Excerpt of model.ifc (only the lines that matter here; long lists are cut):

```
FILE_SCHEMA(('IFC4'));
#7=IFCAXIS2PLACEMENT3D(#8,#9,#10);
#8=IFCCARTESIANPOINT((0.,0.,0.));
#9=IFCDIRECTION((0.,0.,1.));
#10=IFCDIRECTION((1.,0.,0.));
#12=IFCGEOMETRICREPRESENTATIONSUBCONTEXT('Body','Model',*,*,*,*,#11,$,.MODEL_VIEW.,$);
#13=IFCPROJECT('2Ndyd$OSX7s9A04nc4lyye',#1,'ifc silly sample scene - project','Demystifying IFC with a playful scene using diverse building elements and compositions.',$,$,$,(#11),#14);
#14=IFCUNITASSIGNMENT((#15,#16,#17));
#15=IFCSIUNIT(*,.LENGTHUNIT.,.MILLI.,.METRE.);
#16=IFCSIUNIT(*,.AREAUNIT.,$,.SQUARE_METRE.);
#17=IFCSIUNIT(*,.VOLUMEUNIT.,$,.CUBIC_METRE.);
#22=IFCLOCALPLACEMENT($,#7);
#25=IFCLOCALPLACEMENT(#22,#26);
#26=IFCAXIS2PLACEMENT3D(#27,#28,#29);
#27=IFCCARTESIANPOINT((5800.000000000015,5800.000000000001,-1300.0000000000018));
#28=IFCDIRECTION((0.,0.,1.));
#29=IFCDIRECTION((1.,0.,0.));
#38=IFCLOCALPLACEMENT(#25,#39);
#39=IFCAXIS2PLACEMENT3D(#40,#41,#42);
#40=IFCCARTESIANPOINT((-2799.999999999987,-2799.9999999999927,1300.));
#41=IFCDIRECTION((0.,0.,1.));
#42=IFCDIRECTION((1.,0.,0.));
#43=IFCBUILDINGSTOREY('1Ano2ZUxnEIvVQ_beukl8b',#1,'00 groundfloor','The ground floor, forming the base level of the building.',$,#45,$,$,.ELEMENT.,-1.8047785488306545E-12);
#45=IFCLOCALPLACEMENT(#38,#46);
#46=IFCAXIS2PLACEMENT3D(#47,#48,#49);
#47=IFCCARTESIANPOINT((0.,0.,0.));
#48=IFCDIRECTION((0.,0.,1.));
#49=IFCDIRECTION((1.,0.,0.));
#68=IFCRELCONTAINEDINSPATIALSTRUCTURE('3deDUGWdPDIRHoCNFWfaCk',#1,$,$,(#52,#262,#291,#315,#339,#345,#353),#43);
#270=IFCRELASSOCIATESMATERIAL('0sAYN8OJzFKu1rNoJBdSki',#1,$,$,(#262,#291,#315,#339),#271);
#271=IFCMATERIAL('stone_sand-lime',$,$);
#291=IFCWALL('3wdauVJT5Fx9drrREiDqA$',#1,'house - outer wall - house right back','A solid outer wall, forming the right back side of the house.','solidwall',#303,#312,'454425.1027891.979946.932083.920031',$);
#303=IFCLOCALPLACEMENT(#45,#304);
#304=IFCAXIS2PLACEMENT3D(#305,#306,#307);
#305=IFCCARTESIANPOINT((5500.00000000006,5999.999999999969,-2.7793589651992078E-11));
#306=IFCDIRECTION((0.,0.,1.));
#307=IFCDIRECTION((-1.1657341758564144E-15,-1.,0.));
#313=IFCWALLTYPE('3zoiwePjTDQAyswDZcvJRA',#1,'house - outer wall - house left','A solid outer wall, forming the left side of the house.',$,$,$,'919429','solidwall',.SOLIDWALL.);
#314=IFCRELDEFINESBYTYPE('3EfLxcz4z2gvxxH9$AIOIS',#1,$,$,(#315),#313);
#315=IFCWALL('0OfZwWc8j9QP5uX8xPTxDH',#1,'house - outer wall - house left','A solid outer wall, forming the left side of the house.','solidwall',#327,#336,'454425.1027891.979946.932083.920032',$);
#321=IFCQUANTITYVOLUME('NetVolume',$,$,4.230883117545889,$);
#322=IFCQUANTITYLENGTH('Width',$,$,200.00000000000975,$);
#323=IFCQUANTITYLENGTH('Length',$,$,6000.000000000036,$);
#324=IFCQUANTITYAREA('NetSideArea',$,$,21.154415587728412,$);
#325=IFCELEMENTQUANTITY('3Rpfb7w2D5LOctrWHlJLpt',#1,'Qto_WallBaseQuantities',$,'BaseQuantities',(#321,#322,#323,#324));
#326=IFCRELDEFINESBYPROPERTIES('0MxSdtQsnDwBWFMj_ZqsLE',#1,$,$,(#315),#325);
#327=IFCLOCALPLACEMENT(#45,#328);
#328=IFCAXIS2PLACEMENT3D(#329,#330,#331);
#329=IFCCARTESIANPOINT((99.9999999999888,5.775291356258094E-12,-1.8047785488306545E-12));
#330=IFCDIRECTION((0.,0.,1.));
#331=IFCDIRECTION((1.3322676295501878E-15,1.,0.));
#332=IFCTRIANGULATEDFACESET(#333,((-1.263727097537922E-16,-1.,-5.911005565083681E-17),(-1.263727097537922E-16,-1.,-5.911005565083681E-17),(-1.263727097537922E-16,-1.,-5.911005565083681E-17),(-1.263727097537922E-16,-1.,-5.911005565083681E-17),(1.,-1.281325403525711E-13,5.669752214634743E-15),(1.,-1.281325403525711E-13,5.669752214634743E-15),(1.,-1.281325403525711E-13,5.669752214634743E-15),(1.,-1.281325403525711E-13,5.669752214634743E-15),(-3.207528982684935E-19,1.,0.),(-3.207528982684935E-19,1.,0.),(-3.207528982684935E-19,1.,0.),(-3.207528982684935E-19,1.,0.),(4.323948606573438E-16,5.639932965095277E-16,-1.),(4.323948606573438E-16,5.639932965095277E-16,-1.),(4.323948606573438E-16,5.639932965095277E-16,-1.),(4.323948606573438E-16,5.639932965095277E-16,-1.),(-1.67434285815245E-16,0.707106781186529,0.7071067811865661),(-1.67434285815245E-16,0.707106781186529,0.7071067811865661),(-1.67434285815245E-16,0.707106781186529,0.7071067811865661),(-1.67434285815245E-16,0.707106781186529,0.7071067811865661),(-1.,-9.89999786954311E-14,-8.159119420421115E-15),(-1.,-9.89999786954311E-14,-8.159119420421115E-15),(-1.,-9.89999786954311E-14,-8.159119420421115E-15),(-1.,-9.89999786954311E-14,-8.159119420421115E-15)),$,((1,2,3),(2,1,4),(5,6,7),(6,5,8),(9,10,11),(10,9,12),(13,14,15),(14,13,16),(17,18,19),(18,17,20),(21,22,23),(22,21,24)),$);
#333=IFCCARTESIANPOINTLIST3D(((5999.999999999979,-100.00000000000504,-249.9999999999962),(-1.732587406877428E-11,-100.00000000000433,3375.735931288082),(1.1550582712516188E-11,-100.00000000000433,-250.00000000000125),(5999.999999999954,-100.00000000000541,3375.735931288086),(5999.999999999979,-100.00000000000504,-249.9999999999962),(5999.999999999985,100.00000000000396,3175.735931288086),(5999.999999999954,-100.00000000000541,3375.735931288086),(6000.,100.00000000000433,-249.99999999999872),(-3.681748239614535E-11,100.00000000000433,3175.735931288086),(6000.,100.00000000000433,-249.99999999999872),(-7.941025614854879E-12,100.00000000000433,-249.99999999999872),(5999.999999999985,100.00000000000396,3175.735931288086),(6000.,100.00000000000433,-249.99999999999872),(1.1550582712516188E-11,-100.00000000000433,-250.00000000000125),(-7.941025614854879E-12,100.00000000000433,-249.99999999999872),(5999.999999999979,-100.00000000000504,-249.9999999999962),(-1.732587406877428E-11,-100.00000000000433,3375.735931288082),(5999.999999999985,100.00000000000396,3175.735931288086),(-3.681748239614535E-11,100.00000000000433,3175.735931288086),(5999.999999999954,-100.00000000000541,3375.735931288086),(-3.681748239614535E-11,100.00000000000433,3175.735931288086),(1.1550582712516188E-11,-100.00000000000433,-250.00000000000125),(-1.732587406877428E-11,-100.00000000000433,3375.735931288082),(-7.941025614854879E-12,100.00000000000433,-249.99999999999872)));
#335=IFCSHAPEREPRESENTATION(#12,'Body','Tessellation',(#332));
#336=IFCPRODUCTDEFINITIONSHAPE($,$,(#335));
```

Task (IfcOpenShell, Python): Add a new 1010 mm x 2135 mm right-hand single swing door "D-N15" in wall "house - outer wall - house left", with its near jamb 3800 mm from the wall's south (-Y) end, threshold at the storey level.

```python
import numpy as np
import ifcopenshell
import ifcopenshell.api.feature
import ifcopenshell.api.geometry
import ifcopenshell.api.pset
import ifcopenshell.api.root
import ifcopenshell.api.spatial
import ifcopenshell.geom
import ifcopenshell.util.element
import ifcopenshell.util.placement
import ifcopenshell.util.representation
import ifcopenshell.util.shape
import ifcopenshell.util.unit

model = ifcopenshell.open("model.ifc")
unit_scale = ifcopenshell.util.unit.calculate_unit_scale(model)
area_scale = ifcopenshell.util.unit.calculate_unit_scale(model, "AREAUNIT")
volume_scale = ifcopenshell.util.unit.calculate_unit_scale(model, "VOLUMEUNIT")
settings = ifcopenshell.geom.settings()


def volume(element):
    """Net volume in cubic metres, openings subtracted."""
    shape = ifcopenshell.geom.create_shape(settings, element)
    return ifcopenshell.util.shape.get_volume(shape.geometry)


wall = model.by_guid("0OfZwWc8j9QP5uX8xPTxDH")
storey = ifcopenshell.util.element.get_container(wall, ifc_class="IfcBuildingStorey")
context = ifcopenshell.util.representation.get_context(model, "Model", "Body", "MODEL_VIEW")
before = volume(wall)

width, height, from_end, sill = 1.01, 2.135, 3.8, 0.0  # metres

# The wall runs along its own X axis, and the end named is its -X end.
wall_shape = ifcopenshell.geom.create_shape(settings, wall)
x, y, z = ifcopenshell.util.shape.get_vertices(wall_shape.geometry).T
start = x.min() + from_end
face, thickness = float(y.min()), float(y.max() - y.min())
wall_matrix = ifcopenshell.util.placement.get_local_placement(wall.ObjectPlacement)
level = ifcopenshell.util.placement.get_local_placement(storey.ObjectPlacement)[2, 3]


def in_wall(x, y):
    """Placement at x, y metres in the wall's axes, at sill height."""
    matrix = wall_matrix.copy()
    matrix[:, 3] = wall_matrix @ np.array([x / unit_scale, y / unit_scale, 0.0, 1.0])
    matrix[2, 3] = level + sill / unit_scale
    return matrix


# Opening: a box that overshoots both wall faces by 50 mm.
opening = ifcopenshell.api.root.create_entity(model, ifc_class="IfcOpeningElement", predefined_type="OPENING")
box = ifcopenshell.api.geometry.add_wall_representation(
    model, context=context, length=width, height=height, thickness=thickness + 0.1
)
ifcopenshell.api.geometry.assign_representation(model, product=opening, representation=box)
ifcopenshell.api.geometry.edit_object_placement(model, product=opening, matrix=in_wall(start, face - 0.05), is_si=False)
ifcopenshell.api.feature.add_feature(model, feature=opening, element=wall)

door = ifcopenshell.api.root.create_entity(model, ifc_class="IfcDoor", name="D-N15", predefined_type="DOOR")
door.OverallWidth, door.OverallHeight = width / unit_scale, height / unit_scale
door.OperationType = "SINGLE_SWING_RIGHT"
body = ifcopenshell.api.geometry.add_door_representation(
    model,
    context=context,
    overall_width=door.OverallWidth,
    overall_height=door.OverallHeight,
    operation_type="SINGLE_SWING_RIGHT",
    lining_properties={"LiningDepth": thickness / unit_scale, "ThresholdDepth": thickness / unit_scale},
)
ifcopenshell.api.geometry.assign_representation(model, product=door, representation=body)
ifcopenshell.api.spatial.assign_container(model, products=[door], relating_structure=storey)
ifcopenshell.api.feature.add_filling(model, opening=opening, element=door)

# The lining spans the wall, so the door starts at the wall face.
ifcopenshell.api.geometry.edit_object_placement(model, product=door, matrix=in_wall(start, face), is_si=False)

after = volume(wall)

# Update the wall's stored quantities.
qto = model.by_id(ifcopenshell.util.element.get_pset(wall, "Qto_WallBaseQuantities", should_inherit=False)["id"])
ifcopenshell.api.pset.edit_qto(model, qto=qto, properties={
    "NetVolume": after / volume_scale,
    "NetSideArea": after / thickness / area_scale,
})

print(f"wall volume {before:.3f} -> {after:.3f} m3")

model.write("model_rev.ifc")
```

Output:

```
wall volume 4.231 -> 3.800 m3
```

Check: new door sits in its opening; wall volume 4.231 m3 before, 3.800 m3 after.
